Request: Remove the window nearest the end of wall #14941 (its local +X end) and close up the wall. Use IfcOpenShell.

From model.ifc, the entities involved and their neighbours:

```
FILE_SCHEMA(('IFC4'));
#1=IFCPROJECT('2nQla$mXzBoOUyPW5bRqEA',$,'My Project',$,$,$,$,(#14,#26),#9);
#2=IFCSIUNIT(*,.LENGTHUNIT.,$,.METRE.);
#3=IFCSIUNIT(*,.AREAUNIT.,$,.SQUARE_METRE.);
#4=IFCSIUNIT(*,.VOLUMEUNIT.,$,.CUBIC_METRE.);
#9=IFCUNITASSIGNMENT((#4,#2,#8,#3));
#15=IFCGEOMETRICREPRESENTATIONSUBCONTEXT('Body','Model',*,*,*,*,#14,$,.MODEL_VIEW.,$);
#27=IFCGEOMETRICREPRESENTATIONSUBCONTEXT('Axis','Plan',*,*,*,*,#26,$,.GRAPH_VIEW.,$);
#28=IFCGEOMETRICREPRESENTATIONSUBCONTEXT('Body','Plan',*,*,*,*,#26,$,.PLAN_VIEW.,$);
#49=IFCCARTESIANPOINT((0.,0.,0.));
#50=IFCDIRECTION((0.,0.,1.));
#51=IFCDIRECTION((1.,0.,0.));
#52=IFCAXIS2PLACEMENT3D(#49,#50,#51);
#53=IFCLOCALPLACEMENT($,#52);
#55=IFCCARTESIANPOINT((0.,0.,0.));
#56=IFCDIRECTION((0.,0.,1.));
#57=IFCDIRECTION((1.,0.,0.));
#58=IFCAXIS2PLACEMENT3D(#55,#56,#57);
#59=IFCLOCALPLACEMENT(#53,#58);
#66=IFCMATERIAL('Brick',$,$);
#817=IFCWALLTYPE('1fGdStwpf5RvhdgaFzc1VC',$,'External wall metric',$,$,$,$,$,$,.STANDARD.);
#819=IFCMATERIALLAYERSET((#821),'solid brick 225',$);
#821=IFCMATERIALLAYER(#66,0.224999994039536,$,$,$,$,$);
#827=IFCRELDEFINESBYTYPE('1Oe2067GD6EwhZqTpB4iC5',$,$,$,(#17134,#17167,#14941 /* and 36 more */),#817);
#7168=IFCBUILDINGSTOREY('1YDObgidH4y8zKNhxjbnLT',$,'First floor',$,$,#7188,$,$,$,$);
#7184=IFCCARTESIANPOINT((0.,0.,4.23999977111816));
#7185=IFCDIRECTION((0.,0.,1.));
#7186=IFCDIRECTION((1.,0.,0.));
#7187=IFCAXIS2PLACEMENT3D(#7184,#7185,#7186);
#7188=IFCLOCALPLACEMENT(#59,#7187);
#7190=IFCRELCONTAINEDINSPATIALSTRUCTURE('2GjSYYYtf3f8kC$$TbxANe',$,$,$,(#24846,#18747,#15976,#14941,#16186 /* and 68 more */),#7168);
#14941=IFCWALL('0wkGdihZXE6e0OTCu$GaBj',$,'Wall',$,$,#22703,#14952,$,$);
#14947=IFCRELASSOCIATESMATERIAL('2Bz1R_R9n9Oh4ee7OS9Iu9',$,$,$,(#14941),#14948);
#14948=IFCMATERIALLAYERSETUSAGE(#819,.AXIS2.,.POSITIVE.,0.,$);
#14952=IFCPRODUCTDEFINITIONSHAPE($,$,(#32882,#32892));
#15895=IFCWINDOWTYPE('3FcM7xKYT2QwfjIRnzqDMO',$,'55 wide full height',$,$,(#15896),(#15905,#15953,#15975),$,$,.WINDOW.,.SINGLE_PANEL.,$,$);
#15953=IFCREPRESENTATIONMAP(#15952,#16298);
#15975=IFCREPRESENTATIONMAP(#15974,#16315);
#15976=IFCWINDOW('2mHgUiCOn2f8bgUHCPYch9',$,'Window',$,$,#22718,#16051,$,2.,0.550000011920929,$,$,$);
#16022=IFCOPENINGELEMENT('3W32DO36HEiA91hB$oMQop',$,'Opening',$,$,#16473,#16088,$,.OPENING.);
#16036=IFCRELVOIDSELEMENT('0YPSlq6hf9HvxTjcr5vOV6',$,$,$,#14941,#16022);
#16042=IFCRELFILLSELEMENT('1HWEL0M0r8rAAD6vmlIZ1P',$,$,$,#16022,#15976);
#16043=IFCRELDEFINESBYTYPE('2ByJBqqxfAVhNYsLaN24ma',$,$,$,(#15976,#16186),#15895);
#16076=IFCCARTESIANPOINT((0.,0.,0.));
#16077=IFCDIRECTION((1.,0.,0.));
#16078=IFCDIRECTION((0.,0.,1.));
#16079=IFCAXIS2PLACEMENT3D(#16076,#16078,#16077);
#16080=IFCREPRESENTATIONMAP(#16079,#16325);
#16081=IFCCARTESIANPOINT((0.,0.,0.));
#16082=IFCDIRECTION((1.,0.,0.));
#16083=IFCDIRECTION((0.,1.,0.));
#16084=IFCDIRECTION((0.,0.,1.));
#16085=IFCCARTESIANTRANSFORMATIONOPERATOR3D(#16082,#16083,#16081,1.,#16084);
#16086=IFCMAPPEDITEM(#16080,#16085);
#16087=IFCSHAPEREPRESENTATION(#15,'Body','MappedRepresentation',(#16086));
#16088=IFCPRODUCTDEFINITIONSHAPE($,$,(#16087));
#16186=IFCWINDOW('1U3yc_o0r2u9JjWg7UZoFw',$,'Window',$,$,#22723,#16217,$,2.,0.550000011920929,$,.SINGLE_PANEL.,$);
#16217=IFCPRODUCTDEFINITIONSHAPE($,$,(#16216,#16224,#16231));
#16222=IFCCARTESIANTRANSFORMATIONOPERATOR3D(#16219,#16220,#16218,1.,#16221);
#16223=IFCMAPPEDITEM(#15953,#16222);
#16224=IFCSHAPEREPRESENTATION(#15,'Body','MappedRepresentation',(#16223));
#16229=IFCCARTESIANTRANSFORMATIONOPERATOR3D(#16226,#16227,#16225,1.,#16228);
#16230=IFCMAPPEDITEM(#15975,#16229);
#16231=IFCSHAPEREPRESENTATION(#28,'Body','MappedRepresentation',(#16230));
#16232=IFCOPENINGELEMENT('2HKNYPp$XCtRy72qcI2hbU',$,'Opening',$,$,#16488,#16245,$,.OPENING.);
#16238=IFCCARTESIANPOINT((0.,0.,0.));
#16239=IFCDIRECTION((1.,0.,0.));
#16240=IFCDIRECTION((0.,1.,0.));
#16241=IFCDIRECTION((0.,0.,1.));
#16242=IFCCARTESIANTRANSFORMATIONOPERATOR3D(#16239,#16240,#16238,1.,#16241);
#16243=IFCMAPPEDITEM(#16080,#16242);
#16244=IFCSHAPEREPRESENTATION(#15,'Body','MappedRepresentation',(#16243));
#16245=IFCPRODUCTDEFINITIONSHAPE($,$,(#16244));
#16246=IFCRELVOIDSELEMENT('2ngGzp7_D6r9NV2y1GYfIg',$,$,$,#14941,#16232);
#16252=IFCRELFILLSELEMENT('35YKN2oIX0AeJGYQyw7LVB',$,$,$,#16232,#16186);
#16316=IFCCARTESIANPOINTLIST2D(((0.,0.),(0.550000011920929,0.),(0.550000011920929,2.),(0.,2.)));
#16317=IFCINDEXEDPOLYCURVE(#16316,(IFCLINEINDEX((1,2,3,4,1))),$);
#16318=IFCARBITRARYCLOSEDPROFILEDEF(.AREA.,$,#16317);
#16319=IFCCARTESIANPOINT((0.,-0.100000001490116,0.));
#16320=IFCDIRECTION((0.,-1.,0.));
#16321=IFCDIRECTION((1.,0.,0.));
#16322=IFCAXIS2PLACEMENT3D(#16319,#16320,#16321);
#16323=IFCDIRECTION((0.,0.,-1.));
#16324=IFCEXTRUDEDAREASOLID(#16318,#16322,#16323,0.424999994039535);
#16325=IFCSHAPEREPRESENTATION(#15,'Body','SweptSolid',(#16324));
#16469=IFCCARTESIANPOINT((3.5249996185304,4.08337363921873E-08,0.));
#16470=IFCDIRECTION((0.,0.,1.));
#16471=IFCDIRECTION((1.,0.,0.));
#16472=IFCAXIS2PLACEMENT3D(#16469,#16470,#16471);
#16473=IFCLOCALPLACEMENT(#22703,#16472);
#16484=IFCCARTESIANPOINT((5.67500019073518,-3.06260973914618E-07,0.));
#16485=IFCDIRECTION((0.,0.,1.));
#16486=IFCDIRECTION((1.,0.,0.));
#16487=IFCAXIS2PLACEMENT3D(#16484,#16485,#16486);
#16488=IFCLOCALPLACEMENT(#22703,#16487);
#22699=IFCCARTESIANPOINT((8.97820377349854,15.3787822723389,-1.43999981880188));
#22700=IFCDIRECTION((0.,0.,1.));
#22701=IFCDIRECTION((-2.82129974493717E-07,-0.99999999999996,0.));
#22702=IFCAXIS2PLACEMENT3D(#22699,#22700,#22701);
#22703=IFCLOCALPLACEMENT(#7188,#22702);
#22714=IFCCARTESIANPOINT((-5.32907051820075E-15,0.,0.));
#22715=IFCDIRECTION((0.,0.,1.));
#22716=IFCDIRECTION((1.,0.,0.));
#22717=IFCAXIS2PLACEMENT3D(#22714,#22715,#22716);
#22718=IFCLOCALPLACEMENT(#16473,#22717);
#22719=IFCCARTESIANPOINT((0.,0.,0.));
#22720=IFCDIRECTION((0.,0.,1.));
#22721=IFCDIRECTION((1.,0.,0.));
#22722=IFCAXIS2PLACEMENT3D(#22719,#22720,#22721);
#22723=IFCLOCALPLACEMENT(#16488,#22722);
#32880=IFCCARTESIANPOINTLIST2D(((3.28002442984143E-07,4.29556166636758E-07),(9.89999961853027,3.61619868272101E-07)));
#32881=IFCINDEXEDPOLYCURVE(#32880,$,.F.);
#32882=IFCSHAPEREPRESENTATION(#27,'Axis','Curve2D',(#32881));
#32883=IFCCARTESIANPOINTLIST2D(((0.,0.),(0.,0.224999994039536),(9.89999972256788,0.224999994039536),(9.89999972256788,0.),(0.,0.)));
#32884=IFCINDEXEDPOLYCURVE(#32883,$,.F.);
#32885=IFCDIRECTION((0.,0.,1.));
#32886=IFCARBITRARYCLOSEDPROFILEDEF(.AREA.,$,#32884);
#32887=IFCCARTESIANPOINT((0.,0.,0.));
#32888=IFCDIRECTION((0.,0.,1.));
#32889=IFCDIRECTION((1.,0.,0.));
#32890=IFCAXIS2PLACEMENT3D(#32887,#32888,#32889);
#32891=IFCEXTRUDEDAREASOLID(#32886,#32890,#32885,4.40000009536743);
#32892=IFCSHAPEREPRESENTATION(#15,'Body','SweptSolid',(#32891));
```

```python
import ifcopenshell
import ifcopenshell.api.feature
import ifcopenshell.api.root
import ifcopenshell.geom
import ifcopenshell.util.shape

model = ifcopenshell.open("model.ifc")
settings = ifcopenshell.geom.settings()


def volume(element):
    """Net volume in cubic metres, openings subtracted."""
    shape = ifcopenshell.geom.create_shape(settings, element)
    return ifcopenshell.util.shape.get_volume(shape.geometry)


window = model.by_guid("1U3yc_o0r2u9JjWg7UZoFw")
opening = window.FillsVoids[0].RelatingOpeningElement
wall = opening.VoidsElements[0].RelatingBuildingElement
before = volume(wall)

ifcopenshell.api.root.remove_product(model, product=window)
ifcopenshell.api.feature.remove_feature(model, feature=opening)

after = volume(wall)

print(f"wall volume {before:.3f} -> {after:.3f} m3")

model.write("model-out.ifc")
```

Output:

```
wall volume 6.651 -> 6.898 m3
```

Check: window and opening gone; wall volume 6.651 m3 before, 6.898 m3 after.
